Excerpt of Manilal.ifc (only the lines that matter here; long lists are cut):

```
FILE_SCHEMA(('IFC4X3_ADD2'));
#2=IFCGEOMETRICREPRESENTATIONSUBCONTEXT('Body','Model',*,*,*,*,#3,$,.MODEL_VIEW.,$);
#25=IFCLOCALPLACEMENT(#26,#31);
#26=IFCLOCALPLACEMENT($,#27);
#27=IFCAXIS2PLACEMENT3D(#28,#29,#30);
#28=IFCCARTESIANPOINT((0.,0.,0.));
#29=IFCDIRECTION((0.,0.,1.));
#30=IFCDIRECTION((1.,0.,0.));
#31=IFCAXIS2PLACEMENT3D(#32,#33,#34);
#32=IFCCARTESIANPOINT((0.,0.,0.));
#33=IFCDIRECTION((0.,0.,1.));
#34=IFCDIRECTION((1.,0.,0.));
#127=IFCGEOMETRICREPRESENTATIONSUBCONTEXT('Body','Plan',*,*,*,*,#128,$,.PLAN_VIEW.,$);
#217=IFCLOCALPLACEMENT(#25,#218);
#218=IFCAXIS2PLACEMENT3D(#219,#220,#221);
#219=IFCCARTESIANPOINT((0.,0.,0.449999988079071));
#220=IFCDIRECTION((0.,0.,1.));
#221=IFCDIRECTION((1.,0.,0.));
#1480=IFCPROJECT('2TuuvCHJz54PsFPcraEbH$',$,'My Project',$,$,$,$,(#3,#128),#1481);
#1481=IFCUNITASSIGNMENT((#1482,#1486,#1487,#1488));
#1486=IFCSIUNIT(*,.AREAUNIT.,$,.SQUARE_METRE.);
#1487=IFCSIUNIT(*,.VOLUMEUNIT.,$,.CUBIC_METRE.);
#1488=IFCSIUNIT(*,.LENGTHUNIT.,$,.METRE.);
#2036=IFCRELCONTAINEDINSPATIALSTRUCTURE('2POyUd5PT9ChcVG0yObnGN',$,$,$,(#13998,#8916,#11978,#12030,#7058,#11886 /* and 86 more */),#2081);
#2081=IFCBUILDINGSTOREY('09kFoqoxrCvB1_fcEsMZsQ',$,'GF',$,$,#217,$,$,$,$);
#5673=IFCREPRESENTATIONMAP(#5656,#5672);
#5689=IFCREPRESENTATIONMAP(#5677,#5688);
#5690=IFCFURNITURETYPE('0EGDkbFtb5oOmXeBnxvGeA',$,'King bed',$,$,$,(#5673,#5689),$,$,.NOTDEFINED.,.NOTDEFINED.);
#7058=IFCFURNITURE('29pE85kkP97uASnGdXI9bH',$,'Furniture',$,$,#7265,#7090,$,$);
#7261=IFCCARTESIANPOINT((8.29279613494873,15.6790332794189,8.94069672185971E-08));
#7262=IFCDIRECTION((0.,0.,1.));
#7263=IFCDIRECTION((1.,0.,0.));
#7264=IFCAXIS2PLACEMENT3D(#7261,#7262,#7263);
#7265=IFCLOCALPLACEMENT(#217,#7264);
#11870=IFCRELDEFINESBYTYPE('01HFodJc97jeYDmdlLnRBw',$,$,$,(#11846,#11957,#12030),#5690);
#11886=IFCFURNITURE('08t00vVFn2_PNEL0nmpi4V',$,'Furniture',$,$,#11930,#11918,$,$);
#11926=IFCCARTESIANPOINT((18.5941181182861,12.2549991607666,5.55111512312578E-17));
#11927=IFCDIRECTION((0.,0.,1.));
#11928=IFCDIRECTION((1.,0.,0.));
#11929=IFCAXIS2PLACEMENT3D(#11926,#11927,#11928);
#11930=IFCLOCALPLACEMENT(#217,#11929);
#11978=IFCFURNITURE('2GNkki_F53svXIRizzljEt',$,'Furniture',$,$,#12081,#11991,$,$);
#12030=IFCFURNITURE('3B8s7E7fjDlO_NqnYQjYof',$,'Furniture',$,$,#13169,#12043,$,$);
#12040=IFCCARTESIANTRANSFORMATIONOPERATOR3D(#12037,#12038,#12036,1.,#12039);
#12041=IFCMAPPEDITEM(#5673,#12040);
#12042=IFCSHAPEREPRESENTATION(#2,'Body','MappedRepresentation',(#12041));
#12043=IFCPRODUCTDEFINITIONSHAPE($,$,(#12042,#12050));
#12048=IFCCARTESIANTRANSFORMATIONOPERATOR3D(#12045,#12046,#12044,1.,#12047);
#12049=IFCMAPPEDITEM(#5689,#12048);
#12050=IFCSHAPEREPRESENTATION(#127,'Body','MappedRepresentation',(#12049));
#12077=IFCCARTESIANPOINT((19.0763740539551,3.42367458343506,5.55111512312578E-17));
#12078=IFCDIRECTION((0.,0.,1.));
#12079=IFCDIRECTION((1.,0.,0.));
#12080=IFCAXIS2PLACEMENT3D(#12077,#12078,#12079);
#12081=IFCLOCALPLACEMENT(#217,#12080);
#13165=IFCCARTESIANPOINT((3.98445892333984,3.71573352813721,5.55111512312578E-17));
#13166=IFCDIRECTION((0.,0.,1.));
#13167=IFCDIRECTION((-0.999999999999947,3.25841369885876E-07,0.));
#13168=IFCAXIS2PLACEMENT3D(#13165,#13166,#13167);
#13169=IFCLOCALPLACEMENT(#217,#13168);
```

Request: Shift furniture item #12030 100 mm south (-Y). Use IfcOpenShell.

```python
import ifcopenshell
import ifcopenshell.api.geometry
import ifcopenshell.util.placement
import ifcopenshell.util.unit

model = ifcopenshell.open("Manilal.ifc")
unit_scale = ifcopenshell.util.unit.calculate_unit_scale(model)

item = model.by_guid("3B8s7E7fjDlO_NqnYQjYof")
matrix = ifcopenshell.util.placement.get_local_placement(item.ObjectPlacement)
matrix[1, 3] -= 0.1 / unit_scale
ifcopenshell.api.geometry.edit_object_placement(model, product=item, matrix=matrix, is_si=False)

print(ifcopenshell.util.placement.get_local_placement(item.ObjectPlacement).round(3) + 0.0)

model.write("Manilal_updated.ifc")
```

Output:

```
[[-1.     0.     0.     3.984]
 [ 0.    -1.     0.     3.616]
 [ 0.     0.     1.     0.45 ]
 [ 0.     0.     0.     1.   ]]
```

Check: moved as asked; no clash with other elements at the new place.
